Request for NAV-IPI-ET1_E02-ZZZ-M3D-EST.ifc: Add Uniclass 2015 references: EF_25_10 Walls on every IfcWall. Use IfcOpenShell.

First a look at what the model holds.

```python
import ifcopenshell

model = ifcopenshell.open("NAV-IPI-ET1_E02-ZZZ-M3D-EST.ifc")
print(model.schema)
print("classifications:", [c.Name for c in model.by_type("IfcClassification")])
for ifc_class in ("IfcDoor", "IfcRoof", "IfcStair", "IfcWall", "IfcWindow"):
    print(ifc_class, len(model.by_type(ifc_class)))
```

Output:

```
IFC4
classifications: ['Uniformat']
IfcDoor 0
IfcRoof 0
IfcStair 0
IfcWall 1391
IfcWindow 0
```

```python
import ifcopenshell
import ifcopenshell.api.classification

model = ifcopenshell.open("NAV-IPI-ET1_E02-ZZZ-M3D-EST.ifc")

system = ifcopenshell.api.classification.add_classification(model, classification="Uniclass 2015")

codes = {
    "IfcWall": ("EF_25_10", "Walls"),
}
for ifc_class, (code, name) in codes.items():
    products = model.by_type(ifc_class)
    ifcopenshell.api.classification.add_reference(
        model, products=products, classification=system, identification=code, name=name
    )
    print(code, len(products))

model.write("NAV-IPI-ET1_E02-ZZZ-M3D-EST_v2.ifc")
```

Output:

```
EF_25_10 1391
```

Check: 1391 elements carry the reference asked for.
